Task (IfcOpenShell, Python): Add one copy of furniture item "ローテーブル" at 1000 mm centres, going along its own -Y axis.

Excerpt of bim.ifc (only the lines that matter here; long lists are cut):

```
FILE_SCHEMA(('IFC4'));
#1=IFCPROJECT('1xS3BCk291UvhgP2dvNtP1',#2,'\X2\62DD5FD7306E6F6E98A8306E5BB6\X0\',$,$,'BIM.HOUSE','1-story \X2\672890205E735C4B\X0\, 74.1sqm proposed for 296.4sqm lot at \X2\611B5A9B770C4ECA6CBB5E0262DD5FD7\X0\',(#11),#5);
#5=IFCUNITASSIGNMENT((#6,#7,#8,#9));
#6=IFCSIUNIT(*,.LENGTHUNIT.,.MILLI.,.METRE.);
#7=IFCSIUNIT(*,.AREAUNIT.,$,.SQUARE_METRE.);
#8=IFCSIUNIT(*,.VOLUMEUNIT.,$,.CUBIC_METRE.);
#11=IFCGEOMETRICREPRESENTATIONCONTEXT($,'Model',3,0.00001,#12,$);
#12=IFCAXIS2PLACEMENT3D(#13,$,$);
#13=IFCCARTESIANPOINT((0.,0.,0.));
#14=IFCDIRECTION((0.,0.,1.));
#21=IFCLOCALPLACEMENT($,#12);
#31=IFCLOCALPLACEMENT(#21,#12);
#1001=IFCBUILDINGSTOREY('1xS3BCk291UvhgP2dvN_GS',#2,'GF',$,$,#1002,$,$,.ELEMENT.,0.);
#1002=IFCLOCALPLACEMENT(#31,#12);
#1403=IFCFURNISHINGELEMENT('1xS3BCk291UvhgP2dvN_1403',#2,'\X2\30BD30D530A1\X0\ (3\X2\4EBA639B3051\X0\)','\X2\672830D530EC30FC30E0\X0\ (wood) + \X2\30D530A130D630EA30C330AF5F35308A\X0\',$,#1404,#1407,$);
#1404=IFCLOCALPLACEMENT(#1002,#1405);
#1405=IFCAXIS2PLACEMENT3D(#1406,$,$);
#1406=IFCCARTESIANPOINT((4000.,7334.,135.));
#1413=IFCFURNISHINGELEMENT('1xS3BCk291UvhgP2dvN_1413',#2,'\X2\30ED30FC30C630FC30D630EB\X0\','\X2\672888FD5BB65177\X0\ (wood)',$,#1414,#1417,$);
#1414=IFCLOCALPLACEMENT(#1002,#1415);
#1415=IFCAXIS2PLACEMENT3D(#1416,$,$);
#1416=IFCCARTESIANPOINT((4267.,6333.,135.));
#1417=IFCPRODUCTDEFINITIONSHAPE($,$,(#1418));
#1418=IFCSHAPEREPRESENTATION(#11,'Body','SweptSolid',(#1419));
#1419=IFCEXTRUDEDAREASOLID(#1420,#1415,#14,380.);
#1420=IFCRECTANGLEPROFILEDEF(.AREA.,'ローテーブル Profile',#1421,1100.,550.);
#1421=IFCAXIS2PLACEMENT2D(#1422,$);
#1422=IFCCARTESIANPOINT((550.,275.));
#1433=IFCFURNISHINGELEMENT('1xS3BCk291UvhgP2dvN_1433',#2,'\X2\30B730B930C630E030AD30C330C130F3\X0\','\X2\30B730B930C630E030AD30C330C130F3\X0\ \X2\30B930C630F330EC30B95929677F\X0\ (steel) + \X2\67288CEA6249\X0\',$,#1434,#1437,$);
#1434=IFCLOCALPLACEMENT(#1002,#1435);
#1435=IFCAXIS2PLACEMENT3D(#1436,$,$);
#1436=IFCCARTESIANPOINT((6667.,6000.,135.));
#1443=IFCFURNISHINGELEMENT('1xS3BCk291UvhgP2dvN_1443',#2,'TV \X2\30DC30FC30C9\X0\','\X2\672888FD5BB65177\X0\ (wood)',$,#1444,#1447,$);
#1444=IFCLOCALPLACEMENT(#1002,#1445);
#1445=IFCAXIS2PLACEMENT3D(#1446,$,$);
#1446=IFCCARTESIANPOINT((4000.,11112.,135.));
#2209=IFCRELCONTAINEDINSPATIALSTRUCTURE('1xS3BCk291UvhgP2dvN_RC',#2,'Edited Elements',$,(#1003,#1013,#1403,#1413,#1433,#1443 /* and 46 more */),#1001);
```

```python
import ifcopenshell
import ifcopenshell.api.geometry
import ifcopenshell.api.root
import ifcopenshell.util.element
import ifcopenshell.util.placement

model = ifcopenshell.open("bim.ifc")


def reuse_history(source, copy):
    """copy_class also copies each property set's owner history, people and application; keep the originals."""
    for rel in copy.IsDefinedBy:
        if rel.is_a("IfcRelDefinesByProperties") and (history := rel.RelatingPropertyDefinition.OwnerHistory):
            rel.RelatingPropertyDefinition.OwnerHistory = source.OwnerHistory
            ifcopenshell.util.element.remove_deep2(model, history)


source = model.by_guid("1xS3BCk291UvhgP2dvN_1413")
base = ifcopenshell.util.placement.get_local_placement(source.ObjectPlacement)
step = -base[:3, 1] * 1000.0

for i in range(1, 2):
    copy = ifcopenshell.api.root.copy_class(model, product=source)
    copy.Representation = ifcopenshell.util.element.copy_deep(
        model, source.Representation, exclude=["IfcGeometricRepresentationContext", "IfcRepresentationMap"]
    )
    reuse_history(source, copy)
    matrix = base.copy()
    matrix[:3, 3] += i * step
    print("added at", matrix[:3, 3].round(3) + 0.0)
    ifcopenshell.api.geometry.edit_object_placement(model, product=copy, matrix=matrix, is_si=False)

model.write("bim-out.ifc")
```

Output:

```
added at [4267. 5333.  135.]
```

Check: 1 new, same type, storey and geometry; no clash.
